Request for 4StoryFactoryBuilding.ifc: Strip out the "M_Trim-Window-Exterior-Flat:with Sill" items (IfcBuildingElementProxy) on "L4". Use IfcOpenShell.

First a look at what the model holds.

```python
import ifcopenshell
import ifcopenshell.util.element

model = ifcopenshell.open("4StoryFactoryBuilding.ifc")
print(model.schema)
storey = next(s for s in model.by_type("IfcBuildingStorey") if s.Name == "L4")
proxies = [e for e in ifcopenshell.util.element.get_decomposition(storey) if e.is_a("IfcBuildingElementProxy")]
seen = {}
for e in proxies:
    element_type = ifcopenshell.util.element.get_type(e)
    name = element_type.Name if element_type not in (None, e) else None
    seen[name] = seen.get(name, 0) + 1
for name, count in sorted(seen.items(), key=str):
    print(count, "x", name)
```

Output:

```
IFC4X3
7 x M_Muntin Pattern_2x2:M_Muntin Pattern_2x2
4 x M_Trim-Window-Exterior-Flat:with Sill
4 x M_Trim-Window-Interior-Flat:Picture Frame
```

```python
import ifcopenshell
import ifcopenshell.api.root
import ifcopenshell.util.element

model = ifcopenshell.open("4StoryFactoryBuilding.ifc")

storey = next(s for s in model.by_type("IfcBuildingStorey") if s.Name == "L4")
proxies = [e for e in ifcopenshell.util.element.get_decomposition(storey) if e.is_a("IfcBuildingElementProxy")]
targets = [e for e in proxies if (t := ifcopenshell.util.element.get_type(e)) not in (None, e) and t.Name == "M_Trim-Window-Exterior-Flat:with Sill"]

for e in targets:
    ifcopenshell.api.root.remove_product(model, product=e)
print(len(targets), "removed")

model.write("4StoryFactoryBuilding_v2.ifc")
```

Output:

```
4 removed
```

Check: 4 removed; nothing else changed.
